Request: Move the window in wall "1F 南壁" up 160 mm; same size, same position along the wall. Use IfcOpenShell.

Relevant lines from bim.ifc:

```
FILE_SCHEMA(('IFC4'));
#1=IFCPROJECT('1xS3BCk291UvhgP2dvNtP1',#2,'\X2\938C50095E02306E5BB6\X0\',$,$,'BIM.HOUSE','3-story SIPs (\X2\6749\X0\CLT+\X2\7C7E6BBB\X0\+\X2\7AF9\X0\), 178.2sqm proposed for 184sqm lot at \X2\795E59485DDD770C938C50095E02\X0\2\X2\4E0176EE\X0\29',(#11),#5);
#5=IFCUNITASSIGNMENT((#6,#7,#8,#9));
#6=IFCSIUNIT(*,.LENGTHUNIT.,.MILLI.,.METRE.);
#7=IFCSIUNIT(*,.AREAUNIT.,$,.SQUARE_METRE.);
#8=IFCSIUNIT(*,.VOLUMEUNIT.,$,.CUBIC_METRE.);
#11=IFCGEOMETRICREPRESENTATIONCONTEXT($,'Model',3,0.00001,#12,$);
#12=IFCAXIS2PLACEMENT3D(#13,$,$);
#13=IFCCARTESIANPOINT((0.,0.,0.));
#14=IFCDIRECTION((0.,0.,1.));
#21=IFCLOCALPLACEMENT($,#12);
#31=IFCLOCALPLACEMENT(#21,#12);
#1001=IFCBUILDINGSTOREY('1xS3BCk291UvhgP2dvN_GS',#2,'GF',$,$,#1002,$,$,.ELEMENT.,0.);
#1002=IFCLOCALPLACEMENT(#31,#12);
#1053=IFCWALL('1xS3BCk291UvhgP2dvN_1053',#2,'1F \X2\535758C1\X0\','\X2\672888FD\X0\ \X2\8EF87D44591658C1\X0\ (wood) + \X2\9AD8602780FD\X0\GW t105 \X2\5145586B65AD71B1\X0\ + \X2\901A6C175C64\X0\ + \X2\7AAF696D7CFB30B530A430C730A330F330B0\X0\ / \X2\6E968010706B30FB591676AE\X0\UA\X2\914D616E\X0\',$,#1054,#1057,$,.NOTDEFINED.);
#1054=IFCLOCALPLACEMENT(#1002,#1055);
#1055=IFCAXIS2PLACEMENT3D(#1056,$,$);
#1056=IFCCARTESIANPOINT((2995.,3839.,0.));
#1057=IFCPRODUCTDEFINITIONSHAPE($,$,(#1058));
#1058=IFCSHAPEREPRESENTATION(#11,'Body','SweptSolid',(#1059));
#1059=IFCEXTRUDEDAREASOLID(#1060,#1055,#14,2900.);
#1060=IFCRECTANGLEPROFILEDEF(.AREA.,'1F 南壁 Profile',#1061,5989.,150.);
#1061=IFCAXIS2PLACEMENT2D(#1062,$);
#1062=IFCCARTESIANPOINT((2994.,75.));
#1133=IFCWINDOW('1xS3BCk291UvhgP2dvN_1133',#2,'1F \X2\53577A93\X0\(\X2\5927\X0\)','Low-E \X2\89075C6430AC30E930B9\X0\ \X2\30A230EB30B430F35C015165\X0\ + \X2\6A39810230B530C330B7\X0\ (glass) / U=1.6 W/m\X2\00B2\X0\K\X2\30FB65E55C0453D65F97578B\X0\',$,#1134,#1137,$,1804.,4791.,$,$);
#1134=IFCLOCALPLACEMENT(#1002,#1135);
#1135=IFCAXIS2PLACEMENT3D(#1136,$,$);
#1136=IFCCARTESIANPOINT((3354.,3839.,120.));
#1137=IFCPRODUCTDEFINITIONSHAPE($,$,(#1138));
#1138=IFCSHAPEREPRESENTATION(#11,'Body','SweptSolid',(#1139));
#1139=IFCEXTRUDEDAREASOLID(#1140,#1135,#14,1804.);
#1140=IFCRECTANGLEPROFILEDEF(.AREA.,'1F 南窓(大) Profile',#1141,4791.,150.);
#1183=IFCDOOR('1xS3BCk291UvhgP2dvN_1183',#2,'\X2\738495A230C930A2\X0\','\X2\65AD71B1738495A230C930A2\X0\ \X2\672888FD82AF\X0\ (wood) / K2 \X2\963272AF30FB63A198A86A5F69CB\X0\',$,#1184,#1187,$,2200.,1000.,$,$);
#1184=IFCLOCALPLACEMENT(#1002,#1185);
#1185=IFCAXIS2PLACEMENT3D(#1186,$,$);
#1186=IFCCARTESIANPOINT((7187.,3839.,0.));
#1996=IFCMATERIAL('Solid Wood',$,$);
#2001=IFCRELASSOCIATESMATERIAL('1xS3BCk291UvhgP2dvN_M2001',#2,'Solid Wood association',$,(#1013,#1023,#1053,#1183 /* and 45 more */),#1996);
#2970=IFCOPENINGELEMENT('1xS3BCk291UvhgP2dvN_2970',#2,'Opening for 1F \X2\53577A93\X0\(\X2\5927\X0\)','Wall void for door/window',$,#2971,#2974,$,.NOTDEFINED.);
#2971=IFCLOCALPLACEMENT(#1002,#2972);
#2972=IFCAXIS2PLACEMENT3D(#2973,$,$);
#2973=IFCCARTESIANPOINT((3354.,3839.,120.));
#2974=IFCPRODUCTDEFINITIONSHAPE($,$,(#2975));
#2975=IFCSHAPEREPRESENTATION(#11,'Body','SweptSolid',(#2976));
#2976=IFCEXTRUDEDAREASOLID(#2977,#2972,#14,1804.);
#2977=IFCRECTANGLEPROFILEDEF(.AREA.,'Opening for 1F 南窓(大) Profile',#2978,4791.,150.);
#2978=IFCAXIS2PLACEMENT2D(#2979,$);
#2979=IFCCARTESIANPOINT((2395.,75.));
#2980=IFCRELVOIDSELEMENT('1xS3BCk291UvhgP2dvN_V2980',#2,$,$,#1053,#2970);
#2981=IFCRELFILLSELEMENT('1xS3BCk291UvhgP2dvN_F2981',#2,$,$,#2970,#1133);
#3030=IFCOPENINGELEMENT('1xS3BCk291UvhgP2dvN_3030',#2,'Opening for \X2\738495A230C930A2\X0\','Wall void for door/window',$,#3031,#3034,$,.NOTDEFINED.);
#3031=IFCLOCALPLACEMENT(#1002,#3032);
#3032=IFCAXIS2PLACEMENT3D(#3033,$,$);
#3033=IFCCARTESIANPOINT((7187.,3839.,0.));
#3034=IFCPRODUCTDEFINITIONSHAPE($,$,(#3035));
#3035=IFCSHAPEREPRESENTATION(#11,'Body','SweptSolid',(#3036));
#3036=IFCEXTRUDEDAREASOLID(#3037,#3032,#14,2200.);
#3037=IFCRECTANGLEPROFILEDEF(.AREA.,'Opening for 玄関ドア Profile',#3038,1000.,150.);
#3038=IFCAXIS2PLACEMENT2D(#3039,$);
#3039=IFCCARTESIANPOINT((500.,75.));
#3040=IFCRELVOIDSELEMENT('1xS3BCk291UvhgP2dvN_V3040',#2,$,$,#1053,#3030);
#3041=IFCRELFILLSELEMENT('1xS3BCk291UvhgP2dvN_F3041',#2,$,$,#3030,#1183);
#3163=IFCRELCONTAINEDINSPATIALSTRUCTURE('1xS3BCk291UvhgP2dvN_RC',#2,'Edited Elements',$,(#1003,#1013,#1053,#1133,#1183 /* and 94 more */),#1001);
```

```python
import numpy as np
import ifcopenshell
import ifcopenshell.api.geometry
import ifcopenshell.util.placement
import ifcopenshell.util.unit

model = ifcopenshell.open("bim.ifc")
unit_scale = ifcopenshell.util.unit.calculate_unit_scale(model)

window = model.by_guid("1xS3BCk291UvhgP2dvN_1133")
opening = window.FillsVoids[0].RelatingOpeningElement
dz = 0.16 / unit_scale

shift = np.array([0.0, 0.0, dz])
# The window is not placed relative to its opening, so move both.
for product in (opening, window):
    matrix = ifcopenshell.util.placement.get_local_placement(product.ObjectPlacement)
    matrix[:3, 3] += shift
    ifcopenshell.api.geometry.edit_object_placement(model, product=product, matrix=matrix, is_si=False)

print(f"moved by {dz * unit_scale:+.3f} m")

model.write("bim_updated.ifc")
```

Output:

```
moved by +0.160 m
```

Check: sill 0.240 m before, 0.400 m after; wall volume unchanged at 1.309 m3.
